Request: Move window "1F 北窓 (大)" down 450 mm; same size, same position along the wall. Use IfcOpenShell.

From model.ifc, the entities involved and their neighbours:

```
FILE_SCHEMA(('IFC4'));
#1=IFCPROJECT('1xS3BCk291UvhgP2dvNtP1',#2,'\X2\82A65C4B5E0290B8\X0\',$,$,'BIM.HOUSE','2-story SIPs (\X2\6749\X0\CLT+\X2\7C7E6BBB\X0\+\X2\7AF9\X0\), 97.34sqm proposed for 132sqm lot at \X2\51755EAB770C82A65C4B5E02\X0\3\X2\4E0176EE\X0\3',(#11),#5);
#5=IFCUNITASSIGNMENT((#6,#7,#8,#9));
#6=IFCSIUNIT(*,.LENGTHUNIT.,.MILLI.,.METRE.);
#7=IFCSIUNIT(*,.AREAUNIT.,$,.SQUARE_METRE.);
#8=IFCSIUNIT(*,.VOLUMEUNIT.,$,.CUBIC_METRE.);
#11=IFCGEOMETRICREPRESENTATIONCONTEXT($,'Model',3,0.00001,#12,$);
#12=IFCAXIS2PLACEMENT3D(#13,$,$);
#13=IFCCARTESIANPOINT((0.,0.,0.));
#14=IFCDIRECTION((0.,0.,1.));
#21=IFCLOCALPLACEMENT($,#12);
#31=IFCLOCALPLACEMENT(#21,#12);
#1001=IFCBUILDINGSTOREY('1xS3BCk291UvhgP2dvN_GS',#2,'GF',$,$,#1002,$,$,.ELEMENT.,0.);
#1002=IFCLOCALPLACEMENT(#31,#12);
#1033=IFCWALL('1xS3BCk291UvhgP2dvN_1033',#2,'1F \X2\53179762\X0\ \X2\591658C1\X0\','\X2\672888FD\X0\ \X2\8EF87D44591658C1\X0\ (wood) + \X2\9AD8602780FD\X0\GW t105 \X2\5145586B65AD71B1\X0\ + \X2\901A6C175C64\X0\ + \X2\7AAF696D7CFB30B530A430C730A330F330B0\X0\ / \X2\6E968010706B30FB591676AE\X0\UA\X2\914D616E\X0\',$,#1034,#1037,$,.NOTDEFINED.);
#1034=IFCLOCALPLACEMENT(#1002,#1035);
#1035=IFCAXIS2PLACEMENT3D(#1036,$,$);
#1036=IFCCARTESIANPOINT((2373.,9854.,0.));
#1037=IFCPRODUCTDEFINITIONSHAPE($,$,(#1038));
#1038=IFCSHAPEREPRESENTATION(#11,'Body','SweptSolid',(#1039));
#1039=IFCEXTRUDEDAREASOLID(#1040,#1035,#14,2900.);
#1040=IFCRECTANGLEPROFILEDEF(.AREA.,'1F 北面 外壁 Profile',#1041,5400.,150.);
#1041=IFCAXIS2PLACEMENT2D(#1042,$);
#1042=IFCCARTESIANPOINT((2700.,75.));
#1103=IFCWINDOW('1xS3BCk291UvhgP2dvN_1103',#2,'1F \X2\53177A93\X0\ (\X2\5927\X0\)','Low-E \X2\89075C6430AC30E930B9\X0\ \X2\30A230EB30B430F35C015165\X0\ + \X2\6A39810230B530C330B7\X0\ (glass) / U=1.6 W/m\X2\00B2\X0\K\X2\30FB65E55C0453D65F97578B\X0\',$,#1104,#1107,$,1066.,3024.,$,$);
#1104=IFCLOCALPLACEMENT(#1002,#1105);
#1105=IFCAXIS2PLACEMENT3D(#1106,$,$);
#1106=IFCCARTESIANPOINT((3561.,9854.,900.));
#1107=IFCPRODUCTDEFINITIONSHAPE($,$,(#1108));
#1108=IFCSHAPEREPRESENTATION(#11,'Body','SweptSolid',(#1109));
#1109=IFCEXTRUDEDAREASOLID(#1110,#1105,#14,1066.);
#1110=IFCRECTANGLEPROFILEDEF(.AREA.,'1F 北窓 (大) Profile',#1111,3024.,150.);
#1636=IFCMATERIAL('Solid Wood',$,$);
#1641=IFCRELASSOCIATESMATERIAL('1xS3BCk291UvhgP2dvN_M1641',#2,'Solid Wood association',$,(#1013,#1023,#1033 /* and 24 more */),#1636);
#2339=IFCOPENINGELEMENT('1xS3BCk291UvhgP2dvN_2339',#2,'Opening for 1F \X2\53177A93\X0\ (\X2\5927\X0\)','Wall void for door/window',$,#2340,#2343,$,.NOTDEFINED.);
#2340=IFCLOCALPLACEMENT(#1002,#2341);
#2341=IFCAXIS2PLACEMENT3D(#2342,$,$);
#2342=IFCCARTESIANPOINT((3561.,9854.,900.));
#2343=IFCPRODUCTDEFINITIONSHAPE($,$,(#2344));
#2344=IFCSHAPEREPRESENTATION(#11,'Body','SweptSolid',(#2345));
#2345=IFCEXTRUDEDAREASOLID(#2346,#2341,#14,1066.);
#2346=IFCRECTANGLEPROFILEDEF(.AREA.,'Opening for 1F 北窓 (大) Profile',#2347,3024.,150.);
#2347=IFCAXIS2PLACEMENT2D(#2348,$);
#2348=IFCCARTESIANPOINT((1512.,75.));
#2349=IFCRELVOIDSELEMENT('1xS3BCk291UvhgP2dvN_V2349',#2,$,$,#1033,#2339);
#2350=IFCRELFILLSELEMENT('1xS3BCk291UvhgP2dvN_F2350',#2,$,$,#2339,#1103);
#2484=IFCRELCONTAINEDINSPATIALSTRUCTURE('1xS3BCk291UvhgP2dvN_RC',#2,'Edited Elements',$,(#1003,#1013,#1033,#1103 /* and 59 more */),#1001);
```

```python
import numpy as np
import ifcopenshell
import ifcopenshell.api.geometry
import ifcopenshell.util.placement
import ifcopenshell.util.unit

model = ifcopenshell.open("model.ifc")
unit_scale = ifcopenshell.util.unit.calculate_unit_scale(model)

window = model.by_guid("1xS3BCk291UvhgP2dvN_1103")
opening = window.FillsVoids[0].RelatingOpeningElement
dz = -0.45 / unit_scale

shift = np.array([0.0, 0.0, dz])
# The window is not placed relative to its opening, so move both.
for product in (opening, window):
    matrix = ifcopenshell.util.placement.get_local_placement(product.ObjectPlacement)
    matrix[:3, 3] += shift
    ifcopenshell.api.geometry.edit_object_placement(model, product=product, matrix=matrix, is_si=False)

print(f"moved by {dz * unit_scale:+.3f} m")

model.write("model_rev.ifc")
```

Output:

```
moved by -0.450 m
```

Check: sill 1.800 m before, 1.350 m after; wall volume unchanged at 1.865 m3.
